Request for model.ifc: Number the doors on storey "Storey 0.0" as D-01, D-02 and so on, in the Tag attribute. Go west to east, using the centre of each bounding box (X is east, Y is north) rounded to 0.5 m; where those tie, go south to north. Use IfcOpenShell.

First a look at what the model holds.

```python
import ifcopenshell
import ifcopenshell.util.element
import ifcopenshell.util.placement

model = ifcopenshell.open("model.ifc")
print(model.schema)
storey = next(s for s in model.by_type("IfcBuildingStorey") if s.Name == "Storey 0.0")
doors = [e for e in ifcopenshell.util.element.get_decomposition(storey) if e.is_a("IfcDoor")]
for e in sorted(doors, key=lambda e: e.id()):
    origin = ifcopenshell.util.placement.get_local_placement(e.ObjectPlacement)[:3, 3]
    print(e.id(), e.Tag, e.Name, origin.round(2) + 0.0, sep=" | ")
```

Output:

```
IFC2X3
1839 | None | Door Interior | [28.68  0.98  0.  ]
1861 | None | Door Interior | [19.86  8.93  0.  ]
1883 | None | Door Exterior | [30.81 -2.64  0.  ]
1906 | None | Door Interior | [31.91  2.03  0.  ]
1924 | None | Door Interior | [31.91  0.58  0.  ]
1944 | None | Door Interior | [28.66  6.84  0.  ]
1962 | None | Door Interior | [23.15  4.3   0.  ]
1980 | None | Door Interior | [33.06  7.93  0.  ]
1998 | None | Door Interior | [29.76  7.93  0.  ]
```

```python
import ifcopenshell
import ifcopenshell.geom
import ifcopenshell.util.element
import ifcopenshell.util.shape

model = ifcopenshell.open("model.ifc")
settings = ifcopenshell.geom.settings()
settings.set("use-world-coords", True)


def centre(element):
    shape = ifcopenshell.geom.create_shape(settings, element)
    return ifcopenshell.util.shape.get_bbox_centroid(shape.geometry)


storey = next(s for s in model.by_type("IfcBuildingStorey") if s.Name == "Storey 0.0")
doors = [e for e in ifcopenshell.util.element.get_decomposition(storey) if e.is_a("IfcDoor")]

# Insertion points can sit at a corner or the storey origin, so sort by the geometry (in metres).
centres = {e: centre(e) for e in doors}
doors.sort(key=lambda e: (round(centres[e][0] / 0.5), centres[e][1]))

for i, e in enumerate(doors, start=1):
    number = f"D-{i:02d}"
    e.Tag = number
    print(e.id(), number)

model.write("model-out.ifc")
```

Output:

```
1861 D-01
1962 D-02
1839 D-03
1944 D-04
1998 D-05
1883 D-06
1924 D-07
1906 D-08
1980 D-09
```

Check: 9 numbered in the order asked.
